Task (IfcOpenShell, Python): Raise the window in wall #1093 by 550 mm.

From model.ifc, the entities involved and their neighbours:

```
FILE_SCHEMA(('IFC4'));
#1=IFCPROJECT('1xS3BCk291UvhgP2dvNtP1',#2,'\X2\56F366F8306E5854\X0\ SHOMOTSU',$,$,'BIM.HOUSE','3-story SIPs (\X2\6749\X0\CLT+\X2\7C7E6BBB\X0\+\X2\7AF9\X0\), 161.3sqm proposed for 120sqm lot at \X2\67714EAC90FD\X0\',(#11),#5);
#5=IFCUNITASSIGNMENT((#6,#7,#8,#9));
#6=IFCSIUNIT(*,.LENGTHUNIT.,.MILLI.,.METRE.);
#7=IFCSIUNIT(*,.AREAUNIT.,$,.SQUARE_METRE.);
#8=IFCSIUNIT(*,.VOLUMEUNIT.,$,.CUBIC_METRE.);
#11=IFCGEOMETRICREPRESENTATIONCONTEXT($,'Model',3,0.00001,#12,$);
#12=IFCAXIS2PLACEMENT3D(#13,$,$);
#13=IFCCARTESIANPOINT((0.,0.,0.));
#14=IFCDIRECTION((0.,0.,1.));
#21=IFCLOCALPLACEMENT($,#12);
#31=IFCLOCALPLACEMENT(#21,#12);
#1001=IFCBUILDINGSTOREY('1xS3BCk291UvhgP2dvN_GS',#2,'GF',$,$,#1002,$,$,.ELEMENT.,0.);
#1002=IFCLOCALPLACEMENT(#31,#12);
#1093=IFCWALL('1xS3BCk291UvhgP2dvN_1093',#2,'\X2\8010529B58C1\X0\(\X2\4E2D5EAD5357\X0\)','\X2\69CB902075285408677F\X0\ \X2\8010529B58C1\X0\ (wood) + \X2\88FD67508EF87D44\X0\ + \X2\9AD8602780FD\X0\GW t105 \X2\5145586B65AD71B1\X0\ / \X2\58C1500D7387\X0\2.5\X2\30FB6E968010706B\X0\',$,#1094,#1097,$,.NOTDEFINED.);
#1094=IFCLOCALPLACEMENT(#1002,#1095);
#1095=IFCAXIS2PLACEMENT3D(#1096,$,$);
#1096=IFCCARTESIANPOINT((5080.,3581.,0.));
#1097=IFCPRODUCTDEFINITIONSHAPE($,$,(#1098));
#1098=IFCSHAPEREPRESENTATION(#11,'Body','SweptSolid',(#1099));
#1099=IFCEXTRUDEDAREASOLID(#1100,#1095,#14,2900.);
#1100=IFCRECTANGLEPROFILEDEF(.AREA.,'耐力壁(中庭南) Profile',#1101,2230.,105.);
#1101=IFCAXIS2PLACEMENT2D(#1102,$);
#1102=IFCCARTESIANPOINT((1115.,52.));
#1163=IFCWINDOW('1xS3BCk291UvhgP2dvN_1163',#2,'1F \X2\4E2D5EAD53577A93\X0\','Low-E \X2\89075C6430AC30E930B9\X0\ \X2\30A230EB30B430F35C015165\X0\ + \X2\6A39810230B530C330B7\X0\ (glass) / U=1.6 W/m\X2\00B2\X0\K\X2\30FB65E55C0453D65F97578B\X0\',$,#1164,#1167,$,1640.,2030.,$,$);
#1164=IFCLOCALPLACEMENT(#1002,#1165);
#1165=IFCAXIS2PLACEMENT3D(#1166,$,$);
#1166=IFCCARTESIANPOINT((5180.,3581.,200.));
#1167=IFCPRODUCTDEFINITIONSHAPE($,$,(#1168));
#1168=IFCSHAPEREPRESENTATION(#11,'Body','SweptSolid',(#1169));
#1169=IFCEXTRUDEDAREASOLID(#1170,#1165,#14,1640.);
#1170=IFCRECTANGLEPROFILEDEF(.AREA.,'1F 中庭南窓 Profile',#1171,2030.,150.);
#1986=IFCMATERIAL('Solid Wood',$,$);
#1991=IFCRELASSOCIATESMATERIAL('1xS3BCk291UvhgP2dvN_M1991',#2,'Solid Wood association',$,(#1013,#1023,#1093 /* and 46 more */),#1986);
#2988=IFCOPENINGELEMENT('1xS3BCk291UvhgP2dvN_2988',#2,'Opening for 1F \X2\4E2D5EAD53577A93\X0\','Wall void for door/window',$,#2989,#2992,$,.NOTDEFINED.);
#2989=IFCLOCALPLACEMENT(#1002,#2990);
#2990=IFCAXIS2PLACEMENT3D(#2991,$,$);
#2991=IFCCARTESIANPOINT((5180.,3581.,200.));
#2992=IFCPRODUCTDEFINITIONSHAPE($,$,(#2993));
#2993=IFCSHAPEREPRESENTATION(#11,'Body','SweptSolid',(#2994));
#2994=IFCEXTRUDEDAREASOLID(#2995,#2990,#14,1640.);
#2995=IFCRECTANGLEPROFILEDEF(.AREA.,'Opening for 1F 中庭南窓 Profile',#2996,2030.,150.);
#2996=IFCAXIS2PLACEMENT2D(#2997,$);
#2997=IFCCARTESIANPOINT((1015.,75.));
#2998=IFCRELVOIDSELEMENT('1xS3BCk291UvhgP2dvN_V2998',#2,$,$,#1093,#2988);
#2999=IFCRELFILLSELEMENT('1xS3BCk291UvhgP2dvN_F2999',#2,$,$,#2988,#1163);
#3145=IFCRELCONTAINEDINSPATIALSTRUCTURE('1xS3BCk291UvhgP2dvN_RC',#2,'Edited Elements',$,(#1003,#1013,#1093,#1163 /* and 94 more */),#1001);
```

```python
import numpy as np
import ifcopenshell
import ifcopenshell.api.geometry
import ifcopenshell.util.placement
import ifcopenshell.util.unit

model = ifcopenshell.open("model.ifc")
unit_scale = ifcopenshell.util.unit.calculate_unit_scale(model)

window = model.by_guid("1xS3BCk291UvhgP2dvN_1163")
opening = window.FillsVoids[0].RelatingOpeningElement
dz = 550.0

shift = np.array([0.0, 0.0, dz])
# The window is not placed relative to its opening, so move both.
for product in (opening, window):
    matrix = ifcopenshell.util.placement.get_local_placement(product.ObjectPlacement)
    matrix[:3, 3] += shift
    ifcopenshell.api.geometry.edit_object_placement(model, product=product, matrix=matrix, is_si=False)

print(f"moved by {dz * unit_scale:+.3f} m")

model.write("model_v2.ifc")
```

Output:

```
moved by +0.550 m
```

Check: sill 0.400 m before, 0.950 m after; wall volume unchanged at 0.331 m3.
